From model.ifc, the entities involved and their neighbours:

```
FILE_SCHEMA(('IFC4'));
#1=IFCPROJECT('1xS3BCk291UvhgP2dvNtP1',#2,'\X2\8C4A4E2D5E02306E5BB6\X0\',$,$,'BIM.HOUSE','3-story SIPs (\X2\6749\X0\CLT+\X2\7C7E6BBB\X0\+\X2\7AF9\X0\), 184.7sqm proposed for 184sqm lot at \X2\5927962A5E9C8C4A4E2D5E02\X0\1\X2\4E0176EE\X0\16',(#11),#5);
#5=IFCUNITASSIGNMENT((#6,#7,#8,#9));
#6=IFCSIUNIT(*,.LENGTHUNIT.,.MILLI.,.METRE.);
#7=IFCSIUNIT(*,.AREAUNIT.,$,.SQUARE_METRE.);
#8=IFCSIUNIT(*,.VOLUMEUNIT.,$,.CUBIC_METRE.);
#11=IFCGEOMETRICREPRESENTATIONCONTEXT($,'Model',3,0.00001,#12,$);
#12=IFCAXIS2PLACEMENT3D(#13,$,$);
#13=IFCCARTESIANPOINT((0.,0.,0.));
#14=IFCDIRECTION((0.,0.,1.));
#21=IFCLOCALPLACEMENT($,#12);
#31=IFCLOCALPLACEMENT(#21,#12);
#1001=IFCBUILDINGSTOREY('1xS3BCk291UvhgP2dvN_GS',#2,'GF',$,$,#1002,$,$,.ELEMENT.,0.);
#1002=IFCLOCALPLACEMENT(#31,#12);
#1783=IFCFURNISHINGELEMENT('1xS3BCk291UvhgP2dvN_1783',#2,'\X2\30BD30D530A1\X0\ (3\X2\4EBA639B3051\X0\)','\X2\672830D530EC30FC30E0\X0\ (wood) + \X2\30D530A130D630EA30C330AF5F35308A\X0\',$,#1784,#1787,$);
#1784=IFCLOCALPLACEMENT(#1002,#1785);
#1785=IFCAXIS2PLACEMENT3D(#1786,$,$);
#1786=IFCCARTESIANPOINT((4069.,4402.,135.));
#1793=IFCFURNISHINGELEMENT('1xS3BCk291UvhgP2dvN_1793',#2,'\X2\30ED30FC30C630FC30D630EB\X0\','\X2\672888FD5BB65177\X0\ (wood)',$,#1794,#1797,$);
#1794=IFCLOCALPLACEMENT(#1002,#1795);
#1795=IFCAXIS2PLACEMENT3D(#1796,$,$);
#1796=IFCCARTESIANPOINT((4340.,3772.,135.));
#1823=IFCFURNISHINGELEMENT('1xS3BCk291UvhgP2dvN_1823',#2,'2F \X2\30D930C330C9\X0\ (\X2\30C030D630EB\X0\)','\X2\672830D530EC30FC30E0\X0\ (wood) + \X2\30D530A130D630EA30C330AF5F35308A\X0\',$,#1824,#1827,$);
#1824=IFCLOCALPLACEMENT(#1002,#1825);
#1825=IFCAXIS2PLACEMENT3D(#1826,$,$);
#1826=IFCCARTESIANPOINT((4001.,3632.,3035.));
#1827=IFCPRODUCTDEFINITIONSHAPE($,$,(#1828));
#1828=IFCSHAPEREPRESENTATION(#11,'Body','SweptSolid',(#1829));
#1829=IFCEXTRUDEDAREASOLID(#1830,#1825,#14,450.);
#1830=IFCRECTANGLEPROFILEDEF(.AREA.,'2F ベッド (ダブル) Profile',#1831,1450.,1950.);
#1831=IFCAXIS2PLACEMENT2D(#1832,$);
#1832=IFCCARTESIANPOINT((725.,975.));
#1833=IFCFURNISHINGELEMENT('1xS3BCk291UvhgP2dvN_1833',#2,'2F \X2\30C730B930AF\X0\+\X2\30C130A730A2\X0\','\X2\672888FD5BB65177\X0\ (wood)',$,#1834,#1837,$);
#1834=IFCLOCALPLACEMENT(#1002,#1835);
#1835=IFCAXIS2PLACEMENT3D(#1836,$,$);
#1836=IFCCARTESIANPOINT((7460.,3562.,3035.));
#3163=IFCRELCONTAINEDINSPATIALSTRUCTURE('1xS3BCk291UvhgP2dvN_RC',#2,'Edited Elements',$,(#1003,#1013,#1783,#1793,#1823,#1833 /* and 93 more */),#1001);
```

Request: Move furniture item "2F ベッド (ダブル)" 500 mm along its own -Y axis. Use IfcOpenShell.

```python
import ifcopenshell
import ifcopenshell.api.geometry
import ifcopenshell.util.placement
import ifcopenshell.util.unit

model = ifcopenshell.open("model.ifc")
unit_scale = ifcopenshell.util.unit.calculate_unit_scale(model)

item = model.by_guid("1xS3BCk291UvhgP2dvN_1823")
matrix = ifcopenshell.util.placement.get_local_placement(item.ObjectPlacement)
matrix[:3, 3] -= matrix[:3, 1] * 0.5 / unit_scale
ifcopenshell.api.geometry.edit_object_placement(model, product=item, matrix=matrix, is_si=False)

print(ifcopenshell.util.placement.get_local_placement(item.ObjectPlacement).round(3) + 0.0)

model.write("model_updated.ifc")
```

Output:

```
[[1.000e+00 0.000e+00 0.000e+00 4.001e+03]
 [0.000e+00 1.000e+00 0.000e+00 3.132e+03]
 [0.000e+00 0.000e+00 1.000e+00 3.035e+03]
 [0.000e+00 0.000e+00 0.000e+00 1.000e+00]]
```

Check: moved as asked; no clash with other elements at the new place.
